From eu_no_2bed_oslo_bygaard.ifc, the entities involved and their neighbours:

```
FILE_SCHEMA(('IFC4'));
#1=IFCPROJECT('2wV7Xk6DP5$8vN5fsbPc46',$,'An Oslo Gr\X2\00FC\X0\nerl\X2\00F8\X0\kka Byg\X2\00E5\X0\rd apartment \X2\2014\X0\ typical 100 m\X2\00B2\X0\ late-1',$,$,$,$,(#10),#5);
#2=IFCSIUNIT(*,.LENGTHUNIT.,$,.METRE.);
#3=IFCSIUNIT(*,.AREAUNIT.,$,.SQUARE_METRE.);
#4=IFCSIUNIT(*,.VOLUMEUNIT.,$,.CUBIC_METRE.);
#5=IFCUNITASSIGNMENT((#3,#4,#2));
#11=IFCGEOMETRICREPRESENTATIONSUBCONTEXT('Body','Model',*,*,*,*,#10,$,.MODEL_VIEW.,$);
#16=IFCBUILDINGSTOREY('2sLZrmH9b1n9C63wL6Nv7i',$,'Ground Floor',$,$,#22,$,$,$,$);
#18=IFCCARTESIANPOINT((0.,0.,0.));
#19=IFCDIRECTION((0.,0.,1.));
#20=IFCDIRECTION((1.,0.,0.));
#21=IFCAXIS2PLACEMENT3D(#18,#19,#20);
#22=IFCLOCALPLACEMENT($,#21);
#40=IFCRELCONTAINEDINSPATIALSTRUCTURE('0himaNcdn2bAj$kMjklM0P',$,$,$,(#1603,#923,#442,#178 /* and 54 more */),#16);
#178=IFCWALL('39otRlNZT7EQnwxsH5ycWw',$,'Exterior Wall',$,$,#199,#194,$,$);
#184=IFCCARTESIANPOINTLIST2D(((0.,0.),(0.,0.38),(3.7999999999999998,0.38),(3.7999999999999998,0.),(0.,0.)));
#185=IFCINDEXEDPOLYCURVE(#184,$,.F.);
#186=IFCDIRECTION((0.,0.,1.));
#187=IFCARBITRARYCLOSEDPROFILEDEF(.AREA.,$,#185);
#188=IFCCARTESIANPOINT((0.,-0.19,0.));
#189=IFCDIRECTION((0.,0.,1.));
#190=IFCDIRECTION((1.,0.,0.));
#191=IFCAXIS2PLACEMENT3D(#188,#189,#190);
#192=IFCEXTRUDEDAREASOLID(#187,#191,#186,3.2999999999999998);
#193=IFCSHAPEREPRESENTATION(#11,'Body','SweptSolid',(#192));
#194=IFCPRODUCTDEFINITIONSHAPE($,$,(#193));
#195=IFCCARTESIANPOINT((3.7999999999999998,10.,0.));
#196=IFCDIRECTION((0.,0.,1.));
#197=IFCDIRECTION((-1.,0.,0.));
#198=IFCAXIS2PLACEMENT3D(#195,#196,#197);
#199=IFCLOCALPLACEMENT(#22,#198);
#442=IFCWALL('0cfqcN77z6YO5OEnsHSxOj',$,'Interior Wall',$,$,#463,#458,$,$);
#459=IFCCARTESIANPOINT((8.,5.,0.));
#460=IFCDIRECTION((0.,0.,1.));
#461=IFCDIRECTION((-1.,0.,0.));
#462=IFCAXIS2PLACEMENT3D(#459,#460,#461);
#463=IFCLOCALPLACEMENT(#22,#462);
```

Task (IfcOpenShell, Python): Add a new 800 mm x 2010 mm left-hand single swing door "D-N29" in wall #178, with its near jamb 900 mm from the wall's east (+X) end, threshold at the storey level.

```python
import numpy as np
import ifcopenshell
import ifcopenshell.api.feature
import ifcopenshell.api.geometry
import ifcopenshell.api.root
import ifcopenshell.api.spatial
import ifcopenshell.geom
import ifcopenshell.util.element
import ifcopenshell.util.placement
import ifcopenshell.util.representation
import ifcopenshell.util.shape
import ifcopenshell.util.unit

model = ifcopenshell.open("eu_no_2bed_oslo_bygaard.ifc")
unit_scale = ifcopenshell.util.unit.calculate_unit_scale(model)
settings = ifcopenshell.geom.settings()


def volume(element):
    """Net volume in cubic metres, openings subtracted."""
    shape = ifcopenshell.geom.create_shape(settings, element)
    return ifcopenshell.util.shape.get_volume(shape.geometry)


wall = model.by_guid("39otRlNZT7EQnwxsH5ycWw")
storey = ifcopenshell.util.element.get_container(wall, ifc_class="IfcBuildingStorey")
context = ifcopenshell.util.representation.get_context(model, "Model", "Body", "MODEL_VIEW")
before = volume(wall)

width, height, from_end, sill = 0.8, 2.01, 0.9, 0.0  # metres

# The wall runs along its own X axis, and the end named is its -X end.
wall_shape = ifcopenshell.geom.create_shape(settings, wall)
x, y, z = ifcopenshell.util.shape.get_vertices(wall_shape.geometry).T
start = x.min() + from_end
face, thickness = float(y.min()), float(y.max() - y.min())
wall_matrix = ifcopenshell.util.placement.get_local_placement(wall.ObjectPlacement)
level = ifcopenshell.util.placement.get_local_placement(storey.ObjectPlacement)[2, 3]


def in_wall(x, y):
    """Placement at x, y metres in the wall's axes, at sill height."""
    matrix = wall_matrix.copy()
    matrix[:, 3] = wall_matrix @ np.array([x / unit_scale, y / unit_scale, 0.0, 1.0])
    matrix[2, 3] = level + sill / unit_scale
    return matrix


# Opening: a box that overshoots both wall faces by 50 mm.
opening = ifcopenshell.api.root.create_entity(model, ifc_class="IfcOpeningElement", predefined_type="OPENING")
box = ifcopenshell.api.geometry.add_wall_representation(
    model, context=context, length=width, height=height, thickness=thickness + 0.1
)
ifcopenshell.api.geometry.assign_representation(model, product=opening, representation=box)
ifcopenshell.api.geometry.edit_object_placement(model, product=opening, matrix=in_wall(start, face - 0.05), is_si=False)
ifcopenshell.api.feature.add_feature(model, feature=opening, element=wall)

door = ifcopenshell.api.root.create_entity(model, ifc_class="IfcDoor", name="D-N29", predefined_type="DOOR")
door.OverallWidth, door.OverallHeight = width / unit_scale, height / unit_scale
door.OperationType = "SINGLE_SWING_LEFT"
body = ifcopenshell.api.geometry.add_door_representation(
    model,
    context=context,
    overall_width=door.OverallWidth,
    overall_height=door.OverallHeight,
    operation_type="SINGLE_SWING_LEFT",
    lining_properties={"LiningDepth": thickness / unit_scale, "ThresholdDepth": thickness / unit_scale},
)
ifcopenshell.api.geometry.assign_representation(model, product=door, representation=body)
ifcopenshell.api.spatial.assign_container(model, products=[door], relating_structure=storey)
ifcopenshell.api.feature.add_filling(model, opening=opening, element=door)

# The lining spans the wall, so the door starts at the wall face.
ifcopenshell.api.geometry.edit_object_placement(model, product=door, matrix=in_wall(start, face), is_si=False)

after = volume(wall)

print(f"wall volume {before:.3f} -> {after:.3f} m3")

model.write("eu_no_2bed_oslo_bygaard_v2.ifc")
```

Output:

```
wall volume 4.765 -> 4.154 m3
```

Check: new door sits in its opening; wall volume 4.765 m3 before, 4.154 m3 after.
